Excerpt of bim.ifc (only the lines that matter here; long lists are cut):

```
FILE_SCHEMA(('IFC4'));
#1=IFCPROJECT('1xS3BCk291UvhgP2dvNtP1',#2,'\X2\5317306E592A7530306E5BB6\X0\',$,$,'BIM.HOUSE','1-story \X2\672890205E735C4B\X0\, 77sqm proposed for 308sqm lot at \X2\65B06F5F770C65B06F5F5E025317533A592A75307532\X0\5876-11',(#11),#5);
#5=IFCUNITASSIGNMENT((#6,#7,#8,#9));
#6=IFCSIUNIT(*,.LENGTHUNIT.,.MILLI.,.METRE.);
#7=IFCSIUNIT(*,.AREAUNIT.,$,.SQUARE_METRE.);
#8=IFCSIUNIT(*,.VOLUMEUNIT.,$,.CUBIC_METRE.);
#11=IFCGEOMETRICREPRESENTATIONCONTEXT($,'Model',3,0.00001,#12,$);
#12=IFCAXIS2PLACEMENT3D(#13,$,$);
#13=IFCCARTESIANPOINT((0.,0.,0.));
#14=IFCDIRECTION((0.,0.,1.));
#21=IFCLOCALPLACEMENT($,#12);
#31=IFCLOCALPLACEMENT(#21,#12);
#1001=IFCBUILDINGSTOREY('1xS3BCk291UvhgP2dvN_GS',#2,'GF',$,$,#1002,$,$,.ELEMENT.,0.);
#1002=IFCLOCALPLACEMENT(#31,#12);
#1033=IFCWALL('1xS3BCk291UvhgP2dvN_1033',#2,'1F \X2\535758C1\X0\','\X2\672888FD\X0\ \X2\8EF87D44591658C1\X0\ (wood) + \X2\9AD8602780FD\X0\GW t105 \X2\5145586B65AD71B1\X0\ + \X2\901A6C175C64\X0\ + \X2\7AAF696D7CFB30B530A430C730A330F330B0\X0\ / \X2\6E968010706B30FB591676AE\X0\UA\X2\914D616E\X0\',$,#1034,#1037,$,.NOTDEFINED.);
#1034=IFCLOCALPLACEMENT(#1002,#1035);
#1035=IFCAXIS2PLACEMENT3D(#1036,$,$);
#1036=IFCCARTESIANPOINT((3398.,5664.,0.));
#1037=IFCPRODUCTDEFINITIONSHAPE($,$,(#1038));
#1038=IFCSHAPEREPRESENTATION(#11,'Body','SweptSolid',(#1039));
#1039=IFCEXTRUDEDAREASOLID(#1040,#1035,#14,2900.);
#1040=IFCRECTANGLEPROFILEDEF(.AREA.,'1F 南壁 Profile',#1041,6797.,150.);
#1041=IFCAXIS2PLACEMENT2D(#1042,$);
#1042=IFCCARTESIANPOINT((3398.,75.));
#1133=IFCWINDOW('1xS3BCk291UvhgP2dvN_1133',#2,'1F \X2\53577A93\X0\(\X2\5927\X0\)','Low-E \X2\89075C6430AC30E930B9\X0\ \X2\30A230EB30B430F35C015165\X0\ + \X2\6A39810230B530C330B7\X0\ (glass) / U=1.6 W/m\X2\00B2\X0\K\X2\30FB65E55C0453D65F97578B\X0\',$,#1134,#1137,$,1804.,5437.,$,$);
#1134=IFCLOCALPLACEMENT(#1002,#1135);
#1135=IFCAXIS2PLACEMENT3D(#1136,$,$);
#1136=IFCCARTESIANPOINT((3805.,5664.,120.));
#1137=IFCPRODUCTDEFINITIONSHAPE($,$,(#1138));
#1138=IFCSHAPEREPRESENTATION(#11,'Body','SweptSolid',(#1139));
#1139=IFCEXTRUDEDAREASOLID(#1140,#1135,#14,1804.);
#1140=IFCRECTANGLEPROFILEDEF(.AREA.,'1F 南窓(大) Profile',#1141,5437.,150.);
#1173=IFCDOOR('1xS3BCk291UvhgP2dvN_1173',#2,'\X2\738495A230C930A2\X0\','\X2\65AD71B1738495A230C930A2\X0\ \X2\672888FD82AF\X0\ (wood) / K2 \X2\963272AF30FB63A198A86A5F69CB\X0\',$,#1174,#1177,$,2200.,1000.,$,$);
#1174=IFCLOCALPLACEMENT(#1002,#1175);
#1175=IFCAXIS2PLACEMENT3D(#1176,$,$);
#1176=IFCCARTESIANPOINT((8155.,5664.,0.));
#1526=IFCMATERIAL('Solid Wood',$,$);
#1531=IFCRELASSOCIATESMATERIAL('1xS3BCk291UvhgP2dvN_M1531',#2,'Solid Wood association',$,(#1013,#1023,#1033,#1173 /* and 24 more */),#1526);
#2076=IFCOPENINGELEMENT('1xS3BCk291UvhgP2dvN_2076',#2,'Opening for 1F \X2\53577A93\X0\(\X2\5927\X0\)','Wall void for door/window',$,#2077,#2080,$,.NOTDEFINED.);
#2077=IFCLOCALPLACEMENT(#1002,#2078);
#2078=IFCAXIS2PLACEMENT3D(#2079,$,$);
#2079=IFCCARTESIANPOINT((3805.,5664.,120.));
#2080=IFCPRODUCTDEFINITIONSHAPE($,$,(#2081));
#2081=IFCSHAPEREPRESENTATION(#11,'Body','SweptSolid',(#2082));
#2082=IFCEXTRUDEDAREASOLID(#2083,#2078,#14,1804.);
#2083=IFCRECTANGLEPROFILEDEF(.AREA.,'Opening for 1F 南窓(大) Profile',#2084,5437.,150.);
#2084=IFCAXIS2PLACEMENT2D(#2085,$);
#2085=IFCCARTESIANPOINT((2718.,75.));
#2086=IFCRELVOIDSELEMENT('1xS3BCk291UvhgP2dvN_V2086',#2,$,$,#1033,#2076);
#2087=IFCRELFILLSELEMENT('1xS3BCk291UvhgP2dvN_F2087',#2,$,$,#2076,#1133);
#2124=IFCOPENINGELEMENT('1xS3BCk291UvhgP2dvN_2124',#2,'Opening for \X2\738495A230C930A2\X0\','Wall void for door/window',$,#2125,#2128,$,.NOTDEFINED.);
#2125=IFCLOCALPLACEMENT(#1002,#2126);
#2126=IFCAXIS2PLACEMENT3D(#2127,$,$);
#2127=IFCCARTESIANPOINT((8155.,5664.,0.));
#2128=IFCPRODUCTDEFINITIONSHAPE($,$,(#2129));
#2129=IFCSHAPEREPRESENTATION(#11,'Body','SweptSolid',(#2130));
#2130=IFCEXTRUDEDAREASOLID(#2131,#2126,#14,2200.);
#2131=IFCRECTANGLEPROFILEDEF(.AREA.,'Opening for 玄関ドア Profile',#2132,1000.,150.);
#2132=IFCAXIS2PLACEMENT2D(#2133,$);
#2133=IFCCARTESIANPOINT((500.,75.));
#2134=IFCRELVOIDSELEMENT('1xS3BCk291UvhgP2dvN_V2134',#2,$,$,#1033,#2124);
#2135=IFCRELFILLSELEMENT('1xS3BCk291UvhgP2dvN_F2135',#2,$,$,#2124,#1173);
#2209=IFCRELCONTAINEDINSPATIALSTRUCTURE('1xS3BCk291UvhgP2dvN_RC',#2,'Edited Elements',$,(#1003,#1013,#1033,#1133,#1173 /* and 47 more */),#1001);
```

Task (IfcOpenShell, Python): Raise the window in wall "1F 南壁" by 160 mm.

```python
import numpy as np
import ifcopenshell
import ifcopenshell.api.geometry
import ifcopenshell.util.placement
import ifcopenshell.util.unit

model = ifcopenshell.open("bim.ifc")
unit_scale = ifcopenshell.util.unit.calculate_unit_scale(model)

window = model.by_guid("1xS3BCk291UvhgP2dvN_1133")
opening = window.FillsVoids[0].RelatingOpeningElement
dz = 0.16 / unit_scale

shift = np.array([0.0, 0.0, dz])
# The window is not placed relative to its opening, so move both.
for product in (opening, window):
    matrix = ifcopenshell.util.placement.get_local_placement(product.ObjectPlacement)
    matrix[:3, 3] += shift
    ifcopenshell.api.geometry.edit_object_placement(model, product=product, matrix=matrix, is_si=False)

print(f"moved by {dz * unit_scale:+.3f} m")

model.write("bim_v2.ifc")
```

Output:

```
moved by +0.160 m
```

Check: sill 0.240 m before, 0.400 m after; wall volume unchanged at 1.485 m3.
